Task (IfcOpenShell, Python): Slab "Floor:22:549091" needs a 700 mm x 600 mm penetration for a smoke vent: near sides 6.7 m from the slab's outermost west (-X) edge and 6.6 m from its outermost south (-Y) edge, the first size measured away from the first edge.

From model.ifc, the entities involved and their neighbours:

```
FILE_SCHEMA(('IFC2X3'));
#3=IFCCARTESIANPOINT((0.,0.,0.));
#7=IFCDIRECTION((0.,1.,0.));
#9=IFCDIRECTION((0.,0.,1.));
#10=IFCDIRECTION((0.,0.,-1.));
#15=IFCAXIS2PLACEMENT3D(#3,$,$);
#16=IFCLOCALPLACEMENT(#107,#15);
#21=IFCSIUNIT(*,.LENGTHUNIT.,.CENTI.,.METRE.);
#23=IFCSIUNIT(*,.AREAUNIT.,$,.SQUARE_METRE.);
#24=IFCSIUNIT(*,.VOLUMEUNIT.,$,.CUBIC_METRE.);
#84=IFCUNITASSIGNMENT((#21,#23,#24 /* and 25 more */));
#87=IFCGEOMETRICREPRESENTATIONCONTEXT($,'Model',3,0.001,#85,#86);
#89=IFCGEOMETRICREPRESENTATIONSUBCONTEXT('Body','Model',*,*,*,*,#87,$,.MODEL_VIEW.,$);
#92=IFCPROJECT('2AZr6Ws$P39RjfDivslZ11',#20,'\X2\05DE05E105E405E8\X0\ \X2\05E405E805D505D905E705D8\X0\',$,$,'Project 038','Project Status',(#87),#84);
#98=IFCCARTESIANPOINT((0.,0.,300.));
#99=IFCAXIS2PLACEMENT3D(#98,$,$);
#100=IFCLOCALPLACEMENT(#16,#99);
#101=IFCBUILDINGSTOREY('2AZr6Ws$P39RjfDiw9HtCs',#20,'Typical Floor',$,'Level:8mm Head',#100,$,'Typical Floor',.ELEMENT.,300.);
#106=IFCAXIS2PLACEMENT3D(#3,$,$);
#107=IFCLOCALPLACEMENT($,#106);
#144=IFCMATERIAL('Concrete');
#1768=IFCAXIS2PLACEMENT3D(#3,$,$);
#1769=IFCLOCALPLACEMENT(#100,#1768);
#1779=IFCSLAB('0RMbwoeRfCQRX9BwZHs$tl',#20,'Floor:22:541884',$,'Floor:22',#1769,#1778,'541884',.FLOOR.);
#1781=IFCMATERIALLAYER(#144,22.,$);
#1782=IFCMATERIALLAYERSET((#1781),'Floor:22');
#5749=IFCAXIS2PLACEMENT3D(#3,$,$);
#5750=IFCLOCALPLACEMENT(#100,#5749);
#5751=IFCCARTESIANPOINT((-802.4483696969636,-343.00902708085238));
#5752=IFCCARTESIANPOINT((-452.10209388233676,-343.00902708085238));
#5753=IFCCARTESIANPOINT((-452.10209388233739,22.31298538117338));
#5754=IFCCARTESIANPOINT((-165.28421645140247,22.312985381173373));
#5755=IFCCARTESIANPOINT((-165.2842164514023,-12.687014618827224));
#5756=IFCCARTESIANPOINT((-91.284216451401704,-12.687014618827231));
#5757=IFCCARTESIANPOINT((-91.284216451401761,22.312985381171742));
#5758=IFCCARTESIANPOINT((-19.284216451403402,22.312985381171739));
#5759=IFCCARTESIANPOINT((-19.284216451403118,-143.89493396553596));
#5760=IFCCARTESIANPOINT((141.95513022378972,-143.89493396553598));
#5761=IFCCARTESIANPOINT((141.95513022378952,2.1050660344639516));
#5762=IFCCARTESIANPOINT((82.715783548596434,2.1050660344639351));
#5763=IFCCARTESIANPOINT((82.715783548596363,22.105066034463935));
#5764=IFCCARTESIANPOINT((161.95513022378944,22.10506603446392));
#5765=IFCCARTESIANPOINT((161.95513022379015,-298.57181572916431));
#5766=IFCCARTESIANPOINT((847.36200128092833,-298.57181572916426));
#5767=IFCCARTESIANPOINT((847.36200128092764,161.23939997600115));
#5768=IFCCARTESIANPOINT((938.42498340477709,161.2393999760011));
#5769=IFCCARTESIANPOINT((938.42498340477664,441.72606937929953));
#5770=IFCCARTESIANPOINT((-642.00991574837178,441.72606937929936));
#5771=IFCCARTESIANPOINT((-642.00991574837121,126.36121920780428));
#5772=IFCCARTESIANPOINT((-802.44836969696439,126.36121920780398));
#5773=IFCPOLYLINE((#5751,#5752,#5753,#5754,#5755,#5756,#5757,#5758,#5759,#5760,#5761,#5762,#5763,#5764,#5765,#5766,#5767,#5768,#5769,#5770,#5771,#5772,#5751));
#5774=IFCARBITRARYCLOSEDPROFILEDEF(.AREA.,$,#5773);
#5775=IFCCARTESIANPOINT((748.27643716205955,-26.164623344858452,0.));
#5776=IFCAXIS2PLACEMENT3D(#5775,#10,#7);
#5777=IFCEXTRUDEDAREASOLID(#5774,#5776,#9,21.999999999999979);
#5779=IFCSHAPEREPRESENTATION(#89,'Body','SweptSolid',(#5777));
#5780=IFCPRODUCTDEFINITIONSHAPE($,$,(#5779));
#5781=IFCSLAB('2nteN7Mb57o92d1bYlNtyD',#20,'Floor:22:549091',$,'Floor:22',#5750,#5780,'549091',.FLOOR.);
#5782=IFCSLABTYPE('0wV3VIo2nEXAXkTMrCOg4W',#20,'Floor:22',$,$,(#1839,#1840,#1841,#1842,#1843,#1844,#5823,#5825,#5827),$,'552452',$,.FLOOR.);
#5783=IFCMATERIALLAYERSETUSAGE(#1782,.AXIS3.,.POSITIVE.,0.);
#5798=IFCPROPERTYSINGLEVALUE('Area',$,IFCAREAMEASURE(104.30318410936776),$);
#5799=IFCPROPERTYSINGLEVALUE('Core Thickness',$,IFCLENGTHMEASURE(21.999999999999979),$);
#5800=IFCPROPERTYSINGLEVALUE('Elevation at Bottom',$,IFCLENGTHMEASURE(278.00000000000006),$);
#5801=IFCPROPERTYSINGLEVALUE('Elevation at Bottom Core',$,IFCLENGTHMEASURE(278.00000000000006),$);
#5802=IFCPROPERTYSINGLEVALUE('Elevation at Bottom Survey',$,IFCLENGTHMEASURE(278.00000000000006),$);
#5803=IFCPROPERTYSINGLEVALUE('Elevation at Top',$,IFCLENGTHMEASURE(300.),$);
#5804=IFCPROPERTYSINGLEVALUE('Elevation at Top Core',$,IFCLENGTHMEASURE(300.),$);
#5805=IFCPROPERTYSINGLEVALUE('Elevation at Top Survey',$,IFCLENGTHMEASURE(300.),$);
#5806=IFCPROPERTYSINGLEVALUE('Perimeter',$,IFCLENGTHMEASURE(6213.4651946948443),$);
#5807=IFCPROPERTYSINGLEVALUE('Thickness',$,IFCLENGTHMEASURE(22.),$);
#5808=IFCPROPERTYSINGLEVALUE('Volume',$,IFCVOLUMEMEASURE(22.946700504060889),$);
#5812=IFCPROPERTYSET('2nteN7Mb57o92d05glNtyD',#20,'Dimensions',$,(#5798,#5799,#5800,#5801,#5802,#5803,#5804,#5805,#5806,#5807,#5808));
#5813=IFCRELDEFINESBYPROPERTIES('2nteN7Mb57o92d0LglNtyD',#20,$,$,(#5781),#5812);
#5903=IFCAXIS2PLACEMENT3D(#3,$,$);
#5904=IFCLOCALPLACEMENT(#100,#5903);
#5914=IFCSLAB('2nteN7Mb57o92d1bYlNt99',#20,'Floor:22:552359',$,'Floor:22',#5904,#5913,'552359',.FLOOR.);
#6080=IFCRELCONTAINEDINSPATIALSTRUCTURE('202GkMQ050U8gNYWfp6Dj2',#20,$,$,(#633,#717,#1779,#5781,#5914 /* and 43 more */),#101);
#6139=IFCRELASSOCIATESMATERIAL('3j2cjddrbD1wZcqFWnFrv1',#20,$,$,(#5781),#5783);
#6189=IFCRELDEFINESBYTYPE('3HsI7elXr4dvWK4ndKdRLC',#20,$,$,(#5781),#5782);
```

```python
import numpy as np
import ifcopenshell
import ifcopenshell.api.feature
import ifcopenshell.api.geometry
import ifcopenshell.api.pset
import ifcopenshell.api.root
import ifcopenshell.geom
import ifcopenshell.util.element
import ifcopenshell.util.placement
import ifcopenshell.util.representation
import ifcopenshell.util.shape
import ifcopenshell.util.unit

model = ifcopenshell.open("model.ifc")
unit_scale = ifcopenshell.util.unit.calculate_unit_scale(model)
area_scale = ifcopenshell.util.unit.calculate_unit_scale(model, "AREAUNIT")
volume_scale = ifcopenshell.util.unit.calculate_unit_scale(model, "VOLUMEUNIT")
settings = ifcopenshell.geom.settings()


def volume(element):
    """Net volume in cubic metres, openings subtracted."""
    shape = ifcopenshell.geom.create_shape(settings, element)
    return ifcopenshell.util.shape.get_volume(shape.geometry)


slab = model.by_guid("2nteN7Mb57o92d1bYlNtyD")
before = volume(slab)

# Extent in the slab's own axes, in metres. The edges named are its -X and -Y sides.
slab_shape = ifcopenshell.geom.create_shape(settings, slab)
vertices = ifcopenshell.util.shape.get_vertices(slab_shape.geometry)
x_min, y_min, bottom = vertices.min(axis=0)
top = vertices[:, 2].max()

opening = ifcopenshell.api.root.create_entity(model, ifc_class="IfcOpeningElement", name="Smoke vent opening")
context = ifcopenshell.util.representation.get_context(model, "Model", "Body", "MODEL_VIEW")
width, depth = 0.7, 0.6
outline = [(0.0, 0.0), (width, 0.0), (width, depth), (0.0, depth), (0.0, 0.0)]
# Overshoot both faces by 50 mm so the cut is clean.
shape = ifcopenshell.api.geometry.add_slab_representation(
    model, context=context, depth=top - bottom + 0.1, polyline=outline
)
ifcopenshell.api.geometry.assign_representation(model, product=opening, representation=shape)

matrix = ifcopenshell.util.placement.get_local_placement(slab.ObjectPlacement)
matrix[:, 3] = matrix @ np.append(np.array([x_min + 6.7, y_min + 6.6, bottom - 0.05]) / unit_scale, 1.0)
ifcopenshell.api.geometry.edit_object_placement(model, product=opening, matrix=matrix, is_si=False)
ifcopenshell.api.feature.add_feature(model, feature=opening, element=slab)

after = volume(slab)

# Update the slab's stored quantities.
pset = model.by_id(ifcopenshell.util.element.get_pset(slab, "Dimensions", should_inherit=False)["id"])
ifcopenshell.api.pset.edit_pset(model, pset=pset, properties={
    "Area": model.create_entity("IfcAreaMeasure", after / (top - bottom) / area_scale),
    "Volume": model.create_entity("IfcVolumeMeasure", after / volume_scale),
})

print(f"slab volume {before:.3f} -> {after:.3f} m3")

model.write("model_edited.ifc")
```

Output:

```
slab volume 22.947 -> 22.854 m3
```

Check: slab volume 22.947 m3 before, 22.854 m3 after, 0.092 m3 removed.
